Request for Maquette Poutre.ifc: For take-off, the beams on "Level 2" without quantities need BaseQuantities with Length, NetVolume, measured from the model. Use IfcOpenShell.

First a look at what the model holds.

```python
import ifcopenshell
import ifcopenshell.util.element
import ifcopenshell.util.unit

model = ifcopenshell.open("Maquette Poutre.ifc")
print(model.schema)
for unit_type in ("LENGTHUNIT", "AREAUNIT", "VOLUMEUNIT"):
    print(unit_type, ifcopenshell.util.unit.calculate_unit_scale(model, unit_type))
storey = next(s for s in model.by_type("IfcBuildingStorey") if s.Name == "Level 2")
beams = [e for e in ifcopenshell.util.element.get_decomposition(storey) if e.is_a("IfcBeam")]
for e in sorted(beams, key=lambda e: e.id()):
    print(e.id(), e.is_a(), e.Name, list(ifcopenshell.util.element.get_psets(e, qtos_only=True)), sep=" | ")
```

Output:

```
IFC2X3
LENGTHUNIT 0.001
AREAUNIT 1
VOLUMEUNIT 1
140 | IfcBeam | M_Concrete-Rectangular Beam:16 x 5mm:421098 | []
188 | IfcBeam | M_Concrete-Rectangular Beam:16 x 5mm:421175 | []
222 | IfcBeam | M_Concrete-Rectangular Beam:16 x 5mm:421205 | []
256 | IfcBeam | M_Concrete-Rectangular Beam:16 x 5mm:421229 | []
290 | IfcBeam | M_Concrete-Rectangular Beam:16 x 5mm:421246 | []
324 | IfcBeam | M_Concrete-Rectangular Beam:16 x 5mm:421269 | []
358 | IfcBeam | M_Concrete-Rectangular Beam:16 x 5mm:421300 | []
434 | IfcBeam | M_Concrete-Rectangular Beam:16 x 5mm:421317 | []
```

```python
import ifcopenshell
import ifcopenshell.api.pset
import ifcopenshell.geom
import ifcopenshell.util.element
import ifcopenshell.util.shape
import ifcopenshell.util.unit

model = ifcopenshell.open("Maquette Poutre.ifc")
unit_scale = ifcopenshell.util.unit.calculate_unit_scale(model)
volume_scale = ifcopenshell.util.unit.calculate_unit_scale(model, "VOLUMEUNIT")
settings = ifcopenshell.geom.settings()

storey = next(s for s in model.by_type("IfcBuildingStorey") if s.Name == "Level 2")
beams = [e for e in ifcopenshell.util.element.get_decomposition(storey) if e.is_a("IfcBeam")]

for e in sorted(beams, key=lambda e: e.id()):
    if ifcopenshell.util.element.get_psets(e, qtos_only=True, should_inherit=False):
        continue
    # Geometry comes back in metres, in the element's own axes.
    shape = ifcopenshell.geom.create_shape(settings, e)
    values = {
        "Length": ifcopenshell.util.shape.get_max_xyz(shape.geometry) / unit_scale,
        "NetVolume": ifcopenshell.util.shape.get_volume(shape.geometry) / volume_scale,
    }
    qto = ifcopenshell.api.pset.add_qto(model, product=e, name="BaseQuantities")
    ifcopenshell.api.pset.edit_qto(model, qto=qto, properties=values)
    print(e.id(), {k: round(v, 3) for k, v in values.items()})

model.write("Maquette Poutre-out.ifc")
```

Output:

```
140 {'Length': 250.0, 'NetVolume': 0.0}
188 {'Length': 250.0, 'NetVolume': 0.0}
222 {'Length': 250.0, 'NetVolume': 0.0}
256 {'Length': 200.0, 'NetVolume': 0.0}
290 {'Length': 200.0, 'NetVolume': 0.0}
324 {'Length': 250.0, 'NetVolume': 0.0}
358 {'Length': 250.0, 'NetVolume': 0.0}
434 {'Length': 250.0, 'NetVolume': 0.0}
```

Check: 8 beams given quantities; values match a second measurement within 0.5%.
